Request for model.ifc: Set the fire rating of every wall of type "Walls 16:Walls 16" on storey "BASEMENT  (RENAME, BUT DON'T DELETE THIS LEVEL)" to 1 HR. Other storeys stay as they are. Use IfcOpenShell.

First a look at what the model holds.

```python
import ifcopenshell
import ifcopenshell.util.element

model = ifcopenshell.open("model.ifc")
print(model.schema)
storey = next(s for s in model.by_type("IfcBuildingStorey") if s.Name == "BASEMENT  (RENAME, BUT DON'T DELETE THIS LEVEL)")
walls = [e for e in ifcopenshell.util.element.get_decomposition(storey) if e.is_a("IfcWall")]
seen = {}
for e in walls:
    element_type = ifcopenshell.util.element.get_type(e)
    key = (element_type.Name if element_type != e and element_type else None, ifcopenshell.util.element.get_pset(e, "Pset_WallCommon", "FireRating"))
    seen[key] = seen.get(key, 0) + 1
for (name, value), count in sorted(seen.items(), key=str):
    print(count, "x", name, "|", value)
```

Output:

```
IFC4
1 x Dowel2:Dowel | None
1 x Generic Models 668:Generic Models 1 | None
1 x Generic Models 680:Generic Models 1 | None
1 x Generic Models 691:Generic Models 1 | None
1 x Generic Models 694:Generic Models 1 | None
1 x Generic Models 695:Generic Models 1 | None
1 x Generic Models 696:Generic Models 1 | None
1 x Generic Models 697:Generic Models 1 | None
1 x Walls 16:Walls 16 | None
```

```python
import ifcopenshell
import ifcopenshell.api.pset
import ifcopenshell.util.element

model = ifcopenshell.open("model.ifc")

storey = next(s for s in model.by_type("IfcBuildingStorey") if s.Name == "BASEMENT  (RENAME, BUT DON'T DELETE THIS LEVEL)")
walls = [e for e in ifcopenshell.util.element.get_decomposition(storey) if e.is_a("IfcWall")]

count = 0
for e in walls:
    element_type = ifcopenshell.util.element.get_type(e)
    if element_type in (None, e) or element_type.Name != "Walls 16:Walls 16":
        continue
    # add_pset returns the element's existing set when there is one.
    pset = ifcopenshell.api.pset.add_pset(model, product=e, name="Pset_WallCommon")
    ifcopenshell.api.pset.edit_pset(model, pset=pset, properties={"FireRating": "1 HR"})
    count += 1

print(count, "walls updated")

model.write("model_edited.ifc")
```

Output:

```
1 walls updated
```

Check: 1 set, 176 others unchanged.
